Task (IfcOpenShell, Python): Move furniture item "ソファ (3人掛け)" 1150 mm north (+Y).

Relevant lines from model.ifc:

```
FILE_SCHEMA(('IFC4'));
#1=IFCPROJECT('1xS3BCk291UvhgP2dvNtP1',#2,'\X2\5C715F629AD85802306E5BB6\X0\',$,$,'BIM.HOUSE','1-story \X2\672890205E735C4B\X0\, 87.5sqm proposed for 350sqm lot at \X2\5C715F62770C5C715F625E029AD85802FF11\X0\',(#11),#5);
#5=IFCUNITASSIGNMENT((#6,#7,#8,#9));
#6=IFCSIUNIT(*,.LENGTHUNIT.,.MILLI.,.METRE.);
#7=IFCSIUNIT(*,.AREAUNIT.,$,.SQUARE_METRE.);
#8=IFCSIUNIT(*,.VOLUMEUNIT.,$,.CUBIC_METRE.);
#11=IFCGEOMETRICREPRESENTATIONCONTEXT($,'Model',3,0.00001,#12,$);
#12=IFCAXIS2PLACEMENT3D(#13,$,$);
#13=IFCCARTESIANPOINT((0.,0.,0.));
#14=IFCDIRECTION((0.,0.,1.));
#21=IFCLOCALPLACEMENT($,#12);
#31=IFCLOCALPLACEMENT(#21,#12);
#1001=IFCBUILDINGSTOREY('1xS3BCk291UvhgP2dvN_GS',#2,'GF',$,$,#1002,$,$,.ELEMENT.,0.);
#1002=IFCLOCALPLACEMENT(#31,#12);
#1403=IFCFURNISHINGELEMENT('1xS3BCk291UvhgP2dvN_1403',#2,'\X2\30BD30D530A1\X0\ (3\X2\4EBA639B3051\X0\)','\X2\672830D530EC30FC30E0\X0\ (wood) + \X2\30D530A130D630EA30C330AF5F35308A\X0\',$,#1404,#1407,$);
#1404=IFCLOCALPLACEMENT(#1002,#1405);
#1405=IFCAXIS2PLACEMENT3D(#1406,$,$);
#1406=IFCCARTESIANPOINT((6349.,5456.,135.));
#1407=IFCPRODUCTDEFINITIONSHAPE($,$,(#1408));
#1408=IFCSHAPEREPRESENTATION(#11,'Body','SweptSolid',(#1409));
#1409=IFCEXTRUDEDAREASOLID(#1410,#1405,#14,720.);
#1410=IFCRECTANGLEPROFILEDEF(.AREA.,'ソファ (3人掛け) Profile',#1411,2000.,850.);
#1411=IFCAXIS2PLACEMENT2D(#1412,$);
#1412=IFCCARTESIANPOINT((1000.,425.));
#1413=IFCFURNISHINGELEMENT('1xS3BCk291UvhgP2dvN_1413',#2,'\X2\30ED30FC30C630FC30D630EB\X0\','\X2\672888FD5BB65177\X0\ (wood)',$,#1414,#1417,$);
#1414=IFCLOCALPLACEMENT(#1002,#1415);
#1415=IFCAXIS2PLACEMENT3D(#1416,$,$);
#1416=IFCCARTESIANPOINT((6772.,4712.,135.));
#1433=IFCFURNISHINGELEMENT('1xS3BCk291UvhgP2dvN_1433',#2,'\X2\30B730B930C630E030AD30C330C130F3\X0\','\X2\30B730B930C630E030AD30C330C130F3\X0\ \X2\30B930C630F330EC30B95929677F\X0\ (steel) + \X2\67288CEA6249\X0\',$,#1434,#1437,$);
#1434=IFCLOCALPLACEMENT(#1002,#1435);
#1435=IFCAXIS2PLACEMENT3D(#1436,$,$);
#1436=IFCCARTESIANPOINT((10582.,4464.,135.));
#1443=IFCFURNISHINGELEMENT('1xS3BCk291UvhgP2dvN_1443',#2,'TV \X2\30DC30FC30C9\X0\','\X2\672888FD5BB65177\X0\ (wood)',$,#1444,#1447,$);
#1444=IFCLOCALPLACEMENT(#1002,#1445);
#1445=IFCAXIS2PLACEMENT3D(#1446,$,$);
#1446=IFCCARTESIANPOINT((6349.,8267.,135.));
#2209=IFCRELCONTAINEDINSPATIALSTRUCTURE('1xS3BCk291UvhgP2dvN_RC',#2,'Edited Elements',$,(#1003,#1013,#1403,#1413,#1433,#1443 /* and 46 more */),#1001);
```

```python
import ifcopenshell
import ifcopenshell.api.geometry
import ifcopenshell.util.placement
import ifcopenshell.util.unit

model = ifcopenshell.open("model.ifc")
unit_scale = ifcopenshell.util.unit.calculate_unit_scale(model)

item = model.by_guid("1xS3BCk291UvhgP2dvN_1403")
matrix = ifcopenshell.util.placement.get_local_placement(item.ObjectPlacement)
matrix[1, 3] += 1.15 / unit_scale
ifcopenshell.api.geometry.edit_object_placement(model, product=item, matrix=matrix, is_si=False)

print(ifcopenshell.util.placement.get_local_placement(item.ObjectPlacement).round(3) + 0.0)

model.write("model_rev.ifc")
```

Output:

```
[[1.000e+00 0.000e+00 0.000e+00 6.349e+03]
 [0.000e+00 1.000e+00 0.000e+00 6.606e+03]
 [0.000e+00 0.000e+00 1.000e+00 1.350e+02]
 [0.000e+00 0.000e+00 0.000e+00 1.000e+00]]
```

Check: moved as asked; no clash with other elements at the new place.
